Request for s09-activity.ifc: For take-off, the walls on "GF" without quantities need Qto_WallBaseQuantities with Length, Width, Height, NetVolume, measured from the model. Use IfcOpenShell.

First a look at what the model holds.

```python
import ifcopenshell
import ifcopenshell.util.element
import ifcopenshell.util.unit

model = ifcopenshell.open("s09-activity.ifc")
print(model.schema)
for unit_type in ("LENGTHUNIT", "AREAUNIT", "VOLUMEUNIT"):
    print(unit_type, ifcopenshell.util.unit.calculate_unit_scale(model, unit_type))
storey = next(s for s in model.by_type("IfcBuildingStorey") if s.Name == "GF")
walls = [e for e in ifcopenshell.util.element.get_decomposition(storey) if e.is_a("IfcWall")]
for e in sorted(walls, key=lambda e: e.id()):
    print(e.id(), e.is_a(), e.Name, list(ifcopenshell.util.element.get_psets(e, qtos_only=True)), sep=" | ")
```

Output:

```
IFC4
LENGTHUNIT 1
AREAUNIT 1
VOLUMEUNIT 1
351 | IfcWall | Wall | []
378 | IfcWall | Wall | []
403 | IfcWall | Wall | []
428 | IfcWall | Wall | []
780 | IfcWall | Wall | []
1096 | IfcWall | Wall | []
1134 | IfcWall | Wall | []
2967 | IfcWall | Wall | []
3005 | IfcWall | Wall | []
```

```python
import ifcopenshell
import ifcopenshell.api.pset
import ifcopenshell.geom
import ifcopenshell.util.element
import ifcopenshell.util.shape
import ifcopenshell.util.unit

model = ifcopenshell.open("s09-activity.ifc")
unit_scale = ifcopenshell.util.unit.calculate_unit_scale(model)
volume_scale = ifcopenshell.util.unit.calculate_unit_scale(model, "VOLUMEUNIT")
settings = ifcopenshell.geom.settings()

storey = next(s for s in model.by_type("IfcBuildingStorey") if s.Name == "GF")
walls = [e for e in ifcopenshell.util.element.get_decomposition(storey) if e.is_a("IfcWall")]

for e in sorted(walls, key=lambda e: e.id()):
    if ifcopenshell.util.element.get_psets(e, qtos_only=True, should_inherit=False):
        continue
    # Geometry comes back in metres, in the element's own axes.
    shape = ifcopenshell.geom.create_shape(settings, e)
    values = {
        "Length": ifcopenshell.util.shape.get_x(shape.geometry) / unit_scale,
        "Width": ifcopenshell.util.shape.get_y(shape.geometry) / unit_scale,
        "Height": ifcopenshell.util.shape.get_z(shape.geometry) / unit_scale,
        "NetVolume": ifcopenshell.util.shape.get_volume(shape.geometry) / volume_scale,
    }
    qto = ifcopenshell.api.pset.add_qto(model, product=e, name="Qto_WallBaseQuantities")
    ifcopenshell.api.pset.edit_qto(model, qto=qto, properties=values)
    print(e.id(), {k: round(v, 3) for k, v in values.items()})

model.write("s09-activity_rev.ifc")
```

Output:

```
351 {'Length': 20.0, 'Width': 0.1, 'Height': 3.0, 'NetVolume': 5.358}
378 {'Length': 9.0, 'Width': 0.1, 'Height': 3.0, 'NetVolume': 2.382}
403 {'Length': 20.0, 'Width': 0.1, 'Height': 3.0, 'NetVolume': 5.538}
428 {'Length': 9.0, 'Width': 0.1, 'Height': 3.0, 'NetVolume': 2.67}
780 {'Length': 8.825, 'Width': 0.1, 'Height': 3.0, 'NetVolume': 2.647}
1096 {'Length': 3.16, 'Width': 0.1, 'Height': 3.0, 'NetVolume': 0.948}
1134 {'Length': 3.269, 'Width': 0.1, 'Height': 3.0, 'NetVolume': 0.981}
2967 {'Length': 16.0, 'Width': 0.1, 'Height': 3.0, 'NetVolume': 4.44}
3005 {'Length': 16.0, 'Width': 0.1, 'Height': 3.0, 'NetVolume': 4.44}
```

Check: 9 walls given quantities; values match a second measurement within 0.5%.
